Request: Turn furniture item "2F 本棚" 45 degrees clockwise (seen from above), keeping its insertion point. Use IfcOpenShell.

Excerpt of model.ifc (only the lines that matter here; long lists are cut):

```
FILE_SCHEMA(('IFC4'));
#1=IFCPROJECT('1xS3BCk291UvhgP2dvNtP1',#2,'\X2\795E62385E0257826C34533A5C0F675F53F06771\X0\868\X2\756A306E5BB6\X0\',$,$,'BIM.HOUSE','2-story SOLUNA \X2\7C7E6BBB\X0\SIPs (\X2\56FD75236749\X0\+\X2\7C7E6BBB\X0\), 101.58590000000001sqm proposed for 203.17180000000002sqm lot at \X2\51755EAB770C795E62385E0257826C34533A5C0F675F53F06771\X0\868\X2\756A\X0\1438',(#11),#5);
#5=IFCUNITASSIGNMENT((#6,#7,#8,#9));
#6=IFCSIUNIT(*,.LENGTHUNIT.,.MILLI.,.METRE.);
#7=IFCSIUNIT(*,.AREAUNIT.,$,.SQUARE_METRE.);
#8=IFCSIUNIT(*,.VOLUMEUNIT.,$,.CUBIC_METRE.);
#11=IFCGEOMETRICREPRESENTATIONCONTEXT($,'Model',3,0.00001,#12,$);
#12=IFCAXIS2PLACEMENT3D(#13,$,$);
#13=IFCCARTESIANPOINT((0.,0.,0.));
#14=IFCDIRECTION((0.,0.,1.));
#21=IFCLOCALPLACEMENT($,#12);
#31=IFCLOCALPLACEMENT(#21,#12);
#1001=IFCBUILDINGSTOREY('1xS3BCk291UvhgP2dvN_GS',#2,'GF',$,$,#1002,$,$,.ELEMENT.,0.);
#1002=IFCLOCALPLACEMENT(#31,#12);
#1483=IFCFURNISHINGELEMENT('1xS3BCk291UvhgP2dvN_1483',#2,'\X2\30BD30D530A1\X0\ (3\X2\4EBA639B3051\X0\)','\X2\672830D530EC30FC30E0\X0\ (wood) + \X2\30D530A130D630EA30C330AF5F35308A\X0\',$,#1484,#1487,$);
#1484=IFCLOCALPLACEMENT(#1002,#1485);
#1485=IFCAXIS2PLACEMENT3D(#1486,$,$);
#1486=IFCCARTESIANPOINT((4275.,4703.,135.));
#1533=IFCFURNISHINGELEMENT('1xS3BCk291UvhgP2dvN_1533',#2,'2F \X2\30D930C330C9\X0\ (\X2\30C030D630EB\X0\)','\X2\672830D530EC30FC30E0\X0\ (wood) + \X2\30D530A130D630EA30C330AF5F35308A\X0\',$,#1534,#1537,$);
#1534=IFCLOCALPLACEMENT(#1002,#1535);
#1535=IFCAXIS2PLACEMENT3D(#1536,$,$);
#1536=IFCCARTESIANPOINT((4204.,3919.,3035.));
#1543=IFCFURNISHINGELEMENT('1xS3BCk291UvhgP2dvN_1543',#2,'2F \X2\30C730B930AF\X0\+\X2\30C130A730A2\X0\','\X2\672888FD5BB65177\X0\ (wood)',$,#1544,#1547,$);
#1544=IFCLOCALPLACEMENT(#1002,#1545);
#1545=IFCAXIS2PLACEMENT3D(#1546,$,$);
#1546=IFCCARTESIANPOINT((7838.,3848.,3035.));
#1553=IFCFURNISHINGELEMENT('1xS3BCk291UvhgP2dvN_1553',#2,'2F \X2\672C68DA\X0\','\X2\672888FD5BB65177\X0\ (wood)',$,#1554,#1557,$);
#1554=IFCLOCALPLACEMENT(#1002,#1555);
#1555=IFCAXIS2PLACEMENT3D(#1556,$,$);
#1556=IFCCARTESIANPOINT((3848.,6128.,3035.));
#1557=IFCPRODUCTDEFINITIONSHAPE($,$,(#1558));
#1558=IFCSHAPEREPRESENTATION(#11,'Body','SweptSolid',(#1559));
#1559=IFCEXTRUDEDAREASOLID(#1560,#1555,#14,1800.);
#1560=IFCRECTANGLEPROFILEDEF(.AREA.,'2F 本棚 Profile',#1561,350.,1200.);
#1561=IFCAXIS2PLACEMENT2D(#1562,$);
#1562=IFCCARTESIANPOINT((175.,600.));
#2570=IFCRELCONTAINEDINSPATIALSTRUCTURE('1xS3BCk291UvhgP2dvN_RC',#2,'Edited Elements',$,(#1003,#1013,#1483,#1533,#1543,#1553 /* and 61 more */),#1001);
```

```python
import ifcopenshell
import ifcopenshell.api.geometry
import ifcopenshell.util.placement

model = ifcopenshell.open("model.ifc")

item = model.by_id(1553)
matrix = ifcopenshell.util.placement.get_local_placement(item.ObjectPlacement)
matrix = matrix @ ifcopenshell.util.placement.rotation(-45, "Z")
ifcopenshell.api.geometry.edit_object_placement(model, product=item, matrix=matrix, is_si=False)

print(ifcopenshell.util.placement.get_local_placement(item.ObjectPlacement).round(3) + 0.0)

model.write("model_rev.ifc")
```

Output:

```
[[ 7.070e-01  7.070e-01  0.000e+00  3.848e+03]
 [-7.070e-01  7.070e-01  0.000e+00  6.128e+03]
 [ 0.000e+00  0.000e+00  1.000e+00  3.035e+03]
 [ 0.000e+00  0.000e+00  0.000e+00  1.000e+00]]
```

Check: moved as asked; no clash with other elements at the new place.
